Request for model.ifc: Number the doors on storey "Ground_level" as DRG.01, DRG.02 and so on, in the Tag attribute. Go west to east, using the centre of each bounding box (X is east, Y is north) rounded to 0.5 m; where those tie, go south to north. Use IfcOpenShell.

First a look at what the model holds.

```python
import ifcopenshell
import ifcopenshell.util.element
import ifcopenshell.util.placement

model = ifcopenshell.open("model.ifc")
print(model.schema)
storey = next(s for s in model.by_type("IfcBuildingStorey") if s.Name == "Ground_level")
doors = [e for e in ifcopenshell.util.element.get_decomposition(storey) if e.is_a("IfcDoor")]
for e in sorted(doors, key=lambda e: e.id()):
    origin = ifcopenshell.util.placement.get_local_placement(e.ObjectPlacement)[:3, 3]
    print(e.id(), e.Tag, e.Name, origin.round(2) + 0.0, sep=" | ")
```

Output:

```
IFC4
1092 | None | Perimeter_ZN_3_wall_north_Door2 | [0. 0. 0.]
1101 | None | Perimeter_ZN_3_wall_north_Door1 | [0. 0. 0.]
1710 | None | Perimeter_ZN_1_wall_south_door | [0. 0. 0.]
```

```python
import ifcopenshell
import ifcopenshell.geom
import ifcopenshell.util.element
import ifcopenshell.util.shape

model = ifcopenshell.open("model.ifc")
settings = ifcopenshell.geom.settings()
settings.set("use-world-coords", True)


def centre(element):
    shape = ifcopenshell.geom.create_shape(settings, element)
    return ifcopenshell.util.shape.get_bbox_centroid(shape.geometry)


storey = next(s for s in model.by_type("IfcBuildingStorey") if s.Name == "Ground_level")
doors = [e for e in ifcopenshell.util.element.get_decomposition(storey) if e.is_a("IfcDoor")]

# Insertion points can sit at a corner or the storey origin, so sort by the geometry (in metres).
centres = {e: centre(e) for e in doors}
doors.sort(key=lambda e: (round(centres[e][0] / 0.5), centres[e][1]))

for i, e in enumerate(doors, start=1):
    number = f"DRG.{i:02d}"
    e.Tag = number
    print(e.id(), number)

model.write("model_v2.ifc")
```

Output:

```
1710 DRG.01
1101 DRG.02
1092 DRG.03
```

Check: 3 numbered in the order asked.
